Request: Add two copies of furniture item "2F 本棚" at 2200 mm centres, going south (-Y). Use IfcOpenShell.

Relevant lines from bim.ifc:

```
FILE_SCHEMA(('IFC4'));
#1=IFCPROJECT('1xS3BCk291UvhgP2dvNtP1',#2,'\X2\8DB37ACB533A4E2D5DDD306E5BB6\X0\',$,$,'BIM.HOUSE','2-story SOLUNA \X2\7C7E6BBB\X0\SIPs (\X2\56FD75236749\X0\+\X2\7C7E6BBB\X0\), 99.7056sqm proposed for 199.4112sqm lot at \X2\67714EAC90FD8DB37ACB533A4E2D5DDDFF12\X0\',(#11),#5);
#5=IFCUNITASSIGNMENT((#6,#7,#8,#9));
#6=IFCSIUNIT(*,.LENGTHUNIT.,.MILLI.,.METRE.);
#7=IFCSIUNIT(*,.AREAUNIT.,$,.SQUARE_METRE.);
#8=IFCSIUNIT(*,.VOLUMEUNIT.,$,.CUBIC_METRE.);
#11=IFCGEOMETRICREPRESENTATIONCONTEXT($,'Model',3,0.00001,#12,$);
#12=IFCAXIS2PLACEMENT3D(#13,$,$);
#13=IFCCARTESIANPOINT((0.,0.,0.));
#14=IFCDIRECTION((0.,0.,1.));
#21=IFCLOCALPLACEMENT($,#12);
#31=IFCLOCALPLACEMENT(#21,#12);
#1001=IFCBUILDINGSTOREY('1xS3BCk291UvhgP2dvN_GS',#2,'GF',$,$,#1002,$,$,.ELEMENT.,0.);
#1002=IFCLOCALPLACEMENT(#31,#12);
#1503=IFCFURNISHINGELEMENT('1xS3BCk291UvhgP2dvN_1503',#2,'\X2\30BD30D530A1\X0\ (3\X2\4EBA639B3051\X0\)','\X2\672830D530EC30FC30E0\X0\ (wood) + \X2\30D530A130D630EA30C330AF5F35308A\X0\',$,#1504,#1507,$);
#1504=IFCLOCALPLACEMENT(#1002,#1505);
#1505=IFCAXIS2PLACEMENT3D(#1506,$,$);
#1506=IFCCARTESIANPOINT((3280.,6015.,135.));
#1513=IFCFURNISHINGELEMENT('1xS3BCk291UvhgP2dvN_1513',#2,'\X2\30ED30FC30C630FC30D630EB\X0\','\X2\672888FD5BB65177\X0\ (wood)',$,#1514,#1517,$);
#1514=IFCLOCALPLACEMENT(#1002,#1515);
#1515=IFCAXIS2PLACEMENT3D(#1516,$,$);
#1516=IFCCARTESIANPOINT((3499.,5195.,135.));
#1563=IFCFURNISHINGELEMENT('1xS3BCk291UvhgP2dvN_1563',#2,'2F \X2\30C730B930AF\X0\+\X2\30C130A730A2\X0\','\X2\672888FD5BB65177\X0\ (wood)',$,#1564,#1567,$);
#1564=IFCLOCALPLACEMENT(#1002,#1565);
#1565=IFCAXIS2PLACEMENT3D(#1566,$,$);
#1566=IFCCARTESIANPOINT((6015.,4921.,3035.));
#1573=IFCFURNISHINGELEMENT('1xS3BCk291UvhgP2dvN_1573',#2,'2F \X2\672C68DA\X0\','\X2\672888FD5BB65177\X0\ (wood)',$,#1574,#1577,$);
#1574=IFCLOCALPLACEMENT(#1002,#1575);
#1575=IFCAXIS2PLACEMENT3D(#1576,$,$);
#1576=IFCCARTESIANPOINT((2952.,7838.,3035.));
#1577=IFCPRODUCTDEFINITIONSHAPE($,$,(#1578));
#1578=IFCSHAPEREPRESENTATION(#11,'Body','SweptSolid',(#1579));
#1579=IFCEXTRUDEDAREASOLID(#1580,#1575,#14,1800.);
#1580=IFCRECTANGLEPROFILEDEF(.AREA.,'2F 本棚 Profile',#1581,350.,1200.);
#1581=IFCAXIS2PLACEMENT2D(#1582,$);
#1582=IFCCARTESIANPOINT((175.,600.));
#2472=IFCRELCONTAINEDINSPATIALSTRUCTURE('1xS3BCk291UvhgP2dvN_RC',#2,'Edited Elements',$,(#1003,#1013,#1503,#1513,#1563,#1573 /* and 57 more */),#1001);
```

```python
import numpy as np
import ifcopenshell
import ifcopenshell.api.geometry
import ifcopenshell.api.root
import ifcopenshell.util.element
import ifcopenshell.util.placement
import ifcopenshell.util.unit

model = ifcopenshell.open("bim.ifc")
unit_scale = ifcopenshell.util.unit.calculate_unit_scale(model)


def reuse_history(source, copy):
    """copy_class also copies each property set's owner history, people and application; keep the originals."""
    for rel in copy.IsDefinedBy:
        if rel.is_a("IfcRelDefinesByProperties") and (history := rel.RelatingPropertyDefinition.OwnerHistory):
            rel.RelatingPropertyDefinition.OwnerHistory = source.OwnerHistory
            ifcopenshell.util.element.remove_deep2(model, history)


source = model.by_guid("1xS3BCk291UvhgP2dvN_1573")
base = ifcopenshell.util.placement.get_local_placement(source.ObjectPlacement)
step = np.array([0.0, -1.0, 0.0]) * 2.2 / unit_scale

for i in range(1, 3):
    copy = ifcopenshell.api.root.copy_class(model, product=source)
    copy.Representation = ifcopenshell.util.element.copy_deep(
        model, source.Representation, exclude=["IfcGeometricRepresentationContext", "IfcRepresentationMap"]
    )
    reuse_history(source, copy)
    matrix = base.copy()
    matrix[:3, 3] += i * step
    print("added at", matrix[:3, 3].round(3) + 0.0)
    ifcopenshell.api.geometry.edit_object_placement(model, product=copy, matrix=matrix, is_si=False)

model.write("bim_edited.ifc")
```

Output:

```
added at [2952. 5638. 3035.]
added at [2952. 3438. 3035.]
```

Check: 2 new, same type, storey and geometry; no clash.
